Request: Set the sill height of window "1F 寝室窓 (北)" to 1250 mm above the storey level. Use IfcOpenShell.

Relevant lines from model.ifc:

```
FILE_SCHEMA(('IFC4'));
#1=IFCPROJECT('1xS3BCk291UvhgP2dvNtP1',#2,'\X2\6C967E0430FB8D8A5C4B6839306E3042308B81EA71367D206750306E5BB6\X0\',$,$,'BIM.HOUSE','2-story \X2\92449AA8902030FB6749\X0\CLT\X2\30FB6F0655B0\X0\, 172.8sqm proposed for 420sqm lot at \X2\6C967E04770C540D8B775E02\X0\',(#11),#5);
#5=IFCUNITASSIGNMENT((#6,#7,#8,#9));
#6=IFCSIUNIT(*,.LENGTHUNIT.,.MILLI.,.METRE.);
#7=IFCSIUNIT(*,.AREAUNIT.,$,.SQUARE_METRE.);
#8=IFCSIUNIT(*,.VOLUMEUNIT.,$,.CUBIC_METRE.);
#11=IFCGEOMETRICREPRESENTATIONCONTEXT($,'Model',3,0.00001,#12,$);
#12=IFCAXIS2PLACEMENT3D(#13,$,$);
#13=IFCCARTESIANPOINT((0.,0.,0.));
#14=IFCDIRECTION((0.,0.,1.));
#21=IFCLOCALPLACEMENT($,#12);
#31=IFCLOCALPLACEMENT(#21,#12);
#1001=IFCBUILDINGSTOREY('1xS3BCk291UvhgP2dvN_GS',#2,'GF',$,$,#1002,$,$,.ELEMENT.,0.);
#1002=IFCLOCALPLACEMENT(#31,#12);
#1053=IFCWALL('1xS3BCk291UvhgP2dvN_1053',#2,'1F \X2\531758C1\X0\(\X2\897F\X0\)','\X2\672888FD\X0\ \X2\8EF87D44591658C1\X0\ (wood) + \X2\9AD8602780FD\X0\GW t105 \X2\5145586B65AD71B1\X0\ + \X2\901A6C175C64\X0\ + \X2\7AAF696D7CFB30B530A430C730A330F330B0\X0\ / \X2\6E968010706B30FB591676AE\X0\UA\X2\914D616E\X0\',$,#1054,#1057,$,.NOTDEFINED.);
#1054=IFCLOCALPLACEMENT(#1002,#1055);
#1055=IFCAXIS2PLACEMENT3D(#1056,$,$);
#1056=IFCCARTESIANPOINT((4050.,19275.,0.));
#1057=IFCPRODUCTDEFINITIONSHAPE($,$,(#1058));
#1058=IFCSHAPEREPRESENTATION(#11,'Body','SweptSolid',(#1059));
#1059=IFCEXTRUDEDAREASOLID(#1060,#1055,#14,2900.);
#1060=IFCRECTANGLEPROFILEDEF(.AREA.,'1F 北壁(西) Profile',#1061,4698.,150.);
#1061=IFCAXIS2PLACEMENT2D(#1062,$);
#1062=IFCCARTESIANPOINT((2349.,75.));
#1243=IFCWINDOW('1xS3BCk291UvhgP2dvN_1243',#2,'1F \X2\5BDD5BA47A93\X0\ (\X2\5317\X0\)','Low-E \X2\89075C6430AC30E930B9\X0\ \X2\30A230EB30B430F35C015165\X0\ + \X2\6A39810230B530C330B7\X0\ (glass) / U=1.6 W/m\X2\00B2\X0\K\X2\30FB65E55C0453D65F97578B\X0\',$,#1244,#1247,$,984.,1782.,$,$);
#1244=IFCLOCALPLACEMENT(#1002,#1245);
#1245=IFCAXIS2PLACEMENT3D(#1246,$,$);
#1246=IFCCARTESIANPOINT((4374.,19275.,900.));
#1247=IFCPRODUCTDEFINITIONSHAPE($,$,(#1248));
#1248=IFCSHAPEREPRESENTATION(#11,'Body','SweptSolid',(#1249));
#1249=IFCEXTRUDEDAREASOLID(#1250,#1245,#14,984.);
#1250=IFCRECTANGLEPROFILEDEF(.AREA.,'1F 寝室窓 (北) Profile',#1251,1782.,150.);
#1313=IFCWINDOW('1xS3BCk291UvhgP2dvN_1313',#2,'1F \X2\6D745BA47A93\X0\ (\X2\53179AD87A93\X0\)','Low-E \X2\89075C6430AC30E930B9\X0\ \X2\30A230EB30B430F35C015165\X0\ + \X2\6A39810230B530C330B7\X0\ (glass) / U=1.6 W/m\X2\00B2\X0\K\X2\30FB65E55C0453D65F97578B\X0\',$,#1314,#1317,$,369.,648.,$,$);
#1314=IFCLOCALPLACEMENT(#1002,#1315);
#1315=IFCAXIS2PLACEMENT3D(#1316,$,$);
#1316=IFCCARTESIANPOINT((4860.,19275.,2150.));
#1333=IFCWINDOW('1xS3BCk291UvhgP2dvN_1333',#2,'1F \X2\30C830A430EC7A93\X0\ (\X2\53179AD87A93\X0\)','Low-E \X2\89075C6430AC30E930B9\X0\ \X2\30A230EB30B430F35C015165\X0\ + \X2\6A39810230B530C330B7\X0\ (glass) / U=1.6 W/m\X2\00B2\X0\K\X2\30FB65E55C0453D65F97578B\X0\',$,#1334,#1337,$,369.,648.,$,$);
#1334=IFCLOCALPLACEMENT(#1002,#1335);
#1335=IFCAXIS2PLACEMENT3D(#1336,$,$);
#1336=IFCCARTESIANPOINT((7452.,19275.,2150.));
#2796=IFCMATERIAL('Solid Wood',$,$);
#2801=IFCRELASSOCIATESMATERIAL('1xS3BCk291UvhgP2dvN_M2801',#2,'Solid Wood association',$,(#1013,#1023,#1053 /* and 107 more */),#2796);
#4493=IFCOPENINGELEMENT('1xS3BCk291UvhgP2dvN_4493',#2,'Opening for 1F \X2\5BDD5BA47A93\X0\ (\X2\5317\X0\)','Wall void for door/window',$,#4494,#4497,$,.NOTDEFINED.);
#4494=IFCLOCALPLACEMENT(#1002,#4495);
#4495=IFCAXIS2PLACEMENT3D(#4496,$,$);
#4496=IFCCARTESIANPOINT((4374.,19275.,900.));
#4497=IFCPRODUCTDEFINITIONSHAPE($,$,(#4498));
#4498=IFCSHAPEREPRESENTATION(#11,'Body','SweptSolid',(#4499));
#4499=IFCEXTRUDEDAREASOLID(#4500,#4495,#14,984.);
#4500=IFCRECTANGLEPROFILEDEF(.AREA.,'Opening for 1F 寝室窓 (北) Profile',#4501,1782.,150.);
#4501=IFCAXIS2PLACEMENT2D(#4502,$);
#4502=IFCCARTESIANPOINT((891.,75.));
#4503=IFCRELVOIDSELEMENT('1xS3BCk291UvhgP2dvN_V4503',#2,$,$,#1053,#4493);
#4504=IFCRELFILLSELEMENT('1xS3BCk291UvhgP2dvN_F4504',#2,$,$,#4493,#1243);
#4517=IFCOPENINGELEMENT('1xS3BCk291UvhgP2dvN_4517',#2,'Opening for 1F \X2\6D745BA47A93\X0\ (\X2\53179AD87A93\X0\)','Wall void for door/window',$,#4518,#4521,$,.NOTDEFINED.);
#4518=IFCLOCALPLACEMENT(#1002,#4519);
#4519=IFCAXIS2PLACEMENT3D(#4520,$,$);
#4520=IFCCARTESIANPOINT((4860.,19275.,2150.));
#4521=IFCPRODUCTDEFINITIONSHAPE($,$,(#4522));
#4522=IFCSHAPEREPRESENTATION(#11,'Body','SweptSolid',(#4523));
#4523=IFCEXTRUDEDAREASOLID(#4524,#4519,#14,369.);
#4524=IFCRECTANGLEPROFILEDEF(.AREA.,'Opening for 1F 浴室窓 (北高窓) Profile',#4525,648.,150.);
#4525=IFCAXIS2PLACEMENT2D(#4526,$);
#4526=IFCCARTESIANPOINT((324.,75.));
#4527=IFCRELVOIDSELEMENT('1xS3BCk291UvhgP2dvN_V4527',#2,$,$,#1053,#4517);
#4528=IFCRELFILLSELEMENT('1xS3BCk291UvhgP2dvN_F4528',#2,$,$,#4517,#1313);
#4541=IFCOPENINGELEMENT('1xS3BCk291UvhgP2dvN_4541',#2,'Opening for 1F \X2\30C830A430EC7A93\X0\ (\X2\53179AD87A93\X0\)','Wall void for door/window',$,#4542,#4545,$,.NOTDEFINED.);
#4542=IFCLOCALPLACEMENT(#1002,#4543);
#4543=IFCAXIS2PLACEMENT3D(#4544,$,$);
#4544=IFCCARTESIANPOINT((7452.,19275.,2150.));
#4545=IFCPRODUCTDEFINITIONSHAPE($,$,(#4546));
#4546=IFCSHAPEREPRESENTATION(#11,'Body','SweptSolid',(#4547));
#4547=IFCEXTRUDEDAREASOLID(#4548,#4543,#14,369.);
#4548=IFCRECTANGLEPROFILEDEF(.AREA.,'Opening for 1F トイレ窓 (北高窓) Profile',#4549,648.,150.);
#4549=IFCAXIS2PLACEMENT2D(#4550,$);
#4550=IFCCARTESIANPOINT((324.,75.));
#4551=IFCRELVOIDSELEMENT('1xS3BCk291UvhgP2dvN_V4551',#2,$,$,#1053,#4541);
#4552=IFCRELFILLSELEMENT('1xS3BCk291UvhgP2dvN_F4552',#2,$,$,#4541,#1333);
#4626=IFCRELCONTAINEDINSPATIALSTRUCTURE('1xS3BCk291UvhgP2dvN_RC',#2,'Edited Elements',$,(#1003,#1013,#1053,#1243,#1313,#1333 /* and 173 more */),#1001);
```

```python
import numpy as np
import ifcopenshell
import ifcopenshell.api.geometry
import ifcopenshell.geom
import ifcopenshell.util.element
import ifcopenshell.util.placement
import ifcopenshell.util.shape
import ifcopenshell.util.unit

model = ifcopenshell.open("model.ifc")
unit_scale = ifcopenshell.util.unit.calculate_unit_scale(model)

window = model.by_guid("1xS3BCk291UvhgP2dvN_1243")
opening = window.FillsVoids[0].RelatingOpeningElement
storey = ifcopenshell.util.element.get_container(window, ifc_class="IfcBuildingStorey")
level = ifcopenshell.util.placement.get_local_placement(storey.ObjectPlacement)[2, 3]

# The opening's origin need not be at the sill, so measure its lowest point.
shape = ifcopenshell.geom.create_shape(ifcopenshell.geom.settings(), opening)
bottom = ifcopenshell.util.shape.get_shape_bottom_elevation(shape, shape.geometry) / unit_scale
dz = level + 1250.0 - bottom

shift = np.array([0.0, 0.0, dz])
# The window is not placed relative to its opening, so move both.
for product in (opening, window):
    matrix = ifcopenshell.util.placement.get_local_placement(product.ObjectPlacement)
    matrix[:3, 3] += shift
    ifcopenshell.api.geometry.edit_object_placement(model, product=product, matrix=matrix, is_si=False)

print(f"moved by {dz * unit_scale:+.3f} m")

model.write("model-out.ifc")
```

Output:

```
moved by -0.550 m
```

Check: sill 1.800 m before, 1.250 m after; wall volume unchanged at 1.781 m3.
